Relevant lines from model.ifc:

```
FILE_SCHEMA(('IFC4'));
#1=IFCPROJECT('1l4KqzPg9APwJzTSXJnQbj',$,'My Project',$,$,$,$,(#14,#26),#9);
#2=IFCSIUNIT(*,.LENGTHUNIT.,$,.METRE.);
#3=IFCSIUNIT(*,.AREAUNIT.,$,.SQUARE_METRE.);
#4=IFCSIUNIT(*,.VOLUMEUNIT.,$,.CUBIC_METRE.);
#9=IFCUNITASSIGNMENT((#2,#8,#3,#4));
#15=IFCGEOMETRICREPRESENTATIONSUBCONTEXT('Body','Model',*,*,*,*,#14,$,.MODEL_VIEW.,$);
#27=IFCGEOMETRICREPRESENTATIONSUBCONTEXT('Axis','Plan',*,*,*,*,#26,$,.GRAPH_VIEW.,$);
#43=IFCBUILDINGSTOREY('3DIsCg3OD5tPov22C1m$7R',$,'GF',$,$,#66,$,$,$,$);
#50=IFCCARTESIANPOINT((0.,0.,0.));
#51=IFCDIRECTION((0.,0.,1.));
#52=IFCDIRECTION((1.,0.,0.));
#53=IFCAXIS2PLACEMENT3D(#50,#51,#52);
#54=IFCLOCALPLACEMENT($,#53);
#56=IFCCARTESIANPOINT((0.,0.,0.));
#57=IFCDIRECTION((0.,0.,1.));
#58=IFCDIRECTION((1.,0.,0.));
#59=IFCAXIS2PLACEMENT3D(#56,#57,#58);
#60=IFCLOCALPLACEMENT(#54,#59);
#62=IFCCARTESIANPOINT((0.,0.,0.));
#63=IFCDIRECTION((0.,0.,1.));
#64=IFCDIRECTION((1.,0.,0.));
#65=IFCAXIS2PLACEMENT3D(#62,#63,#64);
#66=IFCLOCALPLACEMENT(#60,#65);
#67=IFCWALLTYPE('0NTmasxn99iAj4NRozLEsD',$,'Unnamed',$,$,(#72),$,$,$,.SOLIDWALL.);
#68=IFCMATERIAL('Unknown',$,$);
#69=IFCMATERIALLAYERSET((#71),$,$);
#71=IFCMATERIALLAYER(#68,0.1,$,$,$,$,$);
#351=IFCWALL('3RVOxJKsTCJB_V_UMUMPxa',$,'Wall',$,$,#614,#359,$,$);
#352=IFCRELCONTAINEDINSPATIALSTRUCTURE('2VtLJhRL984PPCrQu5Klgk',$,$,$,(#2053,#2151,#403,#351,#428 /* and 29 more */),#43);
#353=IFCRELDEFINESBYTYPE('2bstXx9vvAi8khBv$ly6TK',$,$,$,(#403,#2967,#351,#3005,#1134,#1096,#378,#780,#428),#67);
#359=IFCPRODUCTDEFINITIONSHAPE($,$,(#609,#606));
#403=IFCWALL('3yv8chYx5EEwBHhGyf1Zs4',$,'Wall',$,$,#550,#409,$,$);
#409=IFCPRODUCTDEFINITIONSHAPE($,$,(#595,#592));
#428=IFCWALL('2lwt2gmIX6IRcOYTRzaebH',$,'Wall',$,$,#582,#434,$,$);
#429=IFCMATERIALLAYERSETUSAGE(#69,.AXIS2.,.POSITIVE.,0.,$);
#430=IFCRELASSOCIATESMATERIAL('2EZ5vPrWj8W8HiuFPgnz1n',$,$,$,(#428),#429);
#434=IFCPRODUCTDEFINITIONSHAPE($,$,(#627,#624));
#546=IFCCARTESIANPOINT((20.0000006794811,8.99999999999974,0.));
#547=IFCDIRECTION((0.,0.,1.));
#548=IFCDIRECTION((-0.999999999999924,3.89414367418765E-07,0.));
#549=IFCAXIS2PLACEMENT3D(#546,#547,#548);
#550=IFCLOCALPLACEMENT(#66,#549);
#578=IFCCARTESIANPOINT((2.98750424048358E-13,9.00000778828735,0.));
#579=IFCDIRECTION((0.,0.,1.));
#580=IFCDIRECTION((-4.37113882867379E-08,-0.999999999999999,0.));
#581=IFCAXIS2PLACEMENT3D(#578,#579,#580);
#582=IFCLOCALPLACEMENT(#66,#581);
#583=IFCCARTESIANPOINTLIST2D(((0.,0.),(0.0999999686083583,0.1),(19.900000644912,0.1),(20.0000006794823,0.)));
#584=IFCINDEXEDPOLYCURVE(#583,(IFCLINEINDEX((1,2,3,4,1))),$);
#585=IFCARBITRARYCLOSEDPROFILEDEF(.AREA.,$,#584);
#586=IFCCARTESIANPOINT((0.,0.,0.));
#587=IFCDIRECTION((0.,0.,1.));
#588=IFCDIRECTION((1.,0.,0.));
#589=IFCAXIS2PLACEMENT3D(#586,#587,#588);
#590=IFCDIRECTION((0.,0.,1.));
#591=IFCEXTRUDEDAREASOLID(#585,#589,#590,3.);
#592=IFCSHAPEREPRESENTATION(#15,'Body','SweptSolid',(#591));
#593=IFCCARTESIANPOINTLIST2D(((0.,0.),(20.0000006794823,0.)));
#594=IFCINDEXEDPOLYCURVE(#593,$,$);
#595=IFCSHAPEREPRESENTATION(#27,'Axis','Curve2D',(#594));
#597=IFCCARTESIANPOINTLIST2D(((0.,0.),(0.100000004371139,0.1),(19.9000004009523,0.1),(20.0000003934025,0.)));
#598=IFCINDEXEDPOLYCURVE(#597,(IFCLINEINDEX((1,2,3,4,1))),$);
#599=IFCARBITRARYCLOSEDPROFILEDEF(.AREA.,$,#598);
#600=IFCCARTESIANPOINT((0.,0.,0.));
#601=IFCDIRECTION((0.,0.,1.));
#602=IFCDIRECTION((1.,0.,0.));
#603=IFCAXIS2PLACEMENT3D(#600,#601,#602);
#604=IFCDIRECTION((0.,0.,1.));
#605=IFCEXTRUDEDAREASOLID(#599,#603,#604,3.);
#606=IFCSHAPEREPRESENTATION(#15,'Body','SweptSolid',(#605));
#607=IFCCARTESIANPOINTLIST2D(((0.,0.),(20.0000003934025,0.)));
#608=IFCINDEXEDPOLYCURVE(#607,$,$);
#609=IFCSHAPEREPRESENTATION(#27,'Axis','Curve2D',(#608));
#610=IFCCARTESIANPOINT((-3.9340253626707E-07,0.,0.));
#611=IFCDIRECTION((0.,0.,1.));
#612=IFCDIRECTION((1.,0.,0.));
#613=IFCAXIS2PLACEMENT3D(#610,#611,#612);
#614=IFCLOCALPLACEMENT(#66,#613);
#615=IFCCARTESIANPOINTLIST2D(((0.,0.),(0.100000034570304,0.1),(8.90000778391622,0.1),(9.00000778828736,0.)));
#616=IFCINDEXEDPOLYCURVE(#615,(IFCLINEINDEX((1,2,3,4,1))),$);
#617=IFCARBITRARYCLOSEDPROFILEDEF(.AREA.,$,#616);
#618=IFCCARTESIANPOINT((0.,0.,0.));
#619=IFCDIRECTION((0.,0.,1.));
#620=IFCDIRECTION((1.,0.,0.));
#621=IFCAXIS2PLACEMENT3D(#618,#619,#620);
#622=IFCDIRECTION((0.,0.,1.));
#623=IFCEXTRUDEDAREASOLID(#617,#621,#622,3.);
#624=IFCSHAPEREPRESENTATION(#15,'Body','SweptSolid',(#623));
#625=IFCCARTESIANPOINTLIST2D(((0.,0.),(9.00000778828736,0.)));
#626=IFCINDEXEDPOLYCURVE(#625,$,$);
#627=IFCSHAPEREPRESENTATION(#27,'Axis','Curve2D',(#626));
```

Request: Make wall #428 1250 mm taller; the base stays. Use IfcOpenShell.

```python
import ifcopenshell
import ifcopenshell.geom
import ifcopenshell.util.representation
import ifcopenshell.util.shape

model = ifcopenshell.open("model.ifc")
settings = ifcopenshell.geom.settings()


def volume(element):
    """Net volume in cubic metres, openings subtracted."""
    shape = ifcopenshell.geom.create_shape(settings, element)
    return ifcopenshell.util.shape.get_volume(shape.geometry)


wall = model.by_guid("2lwt2gmIX6IRcOYTRzaebH")
before = volume(wall)

body = ifcopenshell.util.representation.get_representation(wall, "Model", "Body")
solid = body.Items[0]
old_height = solid.Depth
solid.Depth += 1.25
after = volume(wall)

print(f"height {old_height:g} -> {solid.Depth:g}, volume {before:.3f} -> {after:.3f} m3")

model.write("model_rev.ifc")
```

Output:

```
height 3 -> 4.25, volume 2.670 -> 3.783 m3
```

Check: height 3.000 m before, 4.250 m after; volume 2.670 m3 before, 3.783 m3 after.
